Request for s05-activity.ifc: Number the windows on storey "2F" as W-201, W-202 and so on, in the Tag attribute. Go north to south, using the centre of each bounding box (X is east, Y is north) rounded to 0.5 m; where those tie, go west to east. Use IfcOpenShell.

First a look at what the model holds.

```python
import ifcopenshell
import ifcopenshell.util.element
import ifcopenshell.util.placement

model = ifcopenshell.open("s05-activity.ifc")
print(model.schema)
storey = next(s for s in model.by_type("IfcBuildingStorey") if s.Name == "2F")
windows = [e for e in ifcopenshell.util.element.get_decomposition(storey) if e.is_a("IfcWindow")]
for e in sorted(windows, key=lambda e: e.id()):
    origin = ifcopenshell.util.placement.get_local_placement(e.ObjectPlacement)[:3, 3]
    print(e.id(), e.Tag, e.Name, origin.round(2) + 0.0, sep=" | ")
```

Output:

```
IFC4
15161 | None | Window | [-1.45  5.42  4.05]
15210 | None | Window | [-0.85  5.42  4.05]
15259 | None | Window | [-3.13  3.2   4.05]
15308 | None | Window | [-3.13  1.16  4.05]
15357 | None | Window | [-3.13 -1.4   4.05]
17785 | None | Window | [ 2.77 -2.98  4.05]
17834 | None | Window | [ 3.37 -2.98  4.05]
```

```python
import ifcopenshell
import ifcopenshell.geom
import ifcopenshell.util.element
import ifcopenshell.util.shape

model = ifcopenshell.open("s05-activity.ifc")
settings = ifcopenshell.geom.settings()
settings.set("use-world-coords", True)


def centre(element):
    shape = ifcopenshell.geom.create_shape(settings, element)
    return ifcopenshell.util.shape.get_bbox_centroid(shape.geometry)


storey = next(s for s in model.by_type("IfcBuildingStorey") if s.Name == "2F")
windows = [e for e in ifcopenshell.util.element.get_decomposition(storey) if e.is_a("IfcWindow")]

# Insertion points can sit at a corner or the storey origin, so sort by the geometry (in metres).
centres = {e: centre(e) for e in windows}
windows.sort(key=lambda e: (-round(centres[e][1] / 0.5), centres[e][0]))

for i, e in enumerate(windows, start=1):
    number = f"W-2{i:02d}"
    e.Tag = number
    print(e.id(), number)

model.write("s05-activity_edited.ifc")
```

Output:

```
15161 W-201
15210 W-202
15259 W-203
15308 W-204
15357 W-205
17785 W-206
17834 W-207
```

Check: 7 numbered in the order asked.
